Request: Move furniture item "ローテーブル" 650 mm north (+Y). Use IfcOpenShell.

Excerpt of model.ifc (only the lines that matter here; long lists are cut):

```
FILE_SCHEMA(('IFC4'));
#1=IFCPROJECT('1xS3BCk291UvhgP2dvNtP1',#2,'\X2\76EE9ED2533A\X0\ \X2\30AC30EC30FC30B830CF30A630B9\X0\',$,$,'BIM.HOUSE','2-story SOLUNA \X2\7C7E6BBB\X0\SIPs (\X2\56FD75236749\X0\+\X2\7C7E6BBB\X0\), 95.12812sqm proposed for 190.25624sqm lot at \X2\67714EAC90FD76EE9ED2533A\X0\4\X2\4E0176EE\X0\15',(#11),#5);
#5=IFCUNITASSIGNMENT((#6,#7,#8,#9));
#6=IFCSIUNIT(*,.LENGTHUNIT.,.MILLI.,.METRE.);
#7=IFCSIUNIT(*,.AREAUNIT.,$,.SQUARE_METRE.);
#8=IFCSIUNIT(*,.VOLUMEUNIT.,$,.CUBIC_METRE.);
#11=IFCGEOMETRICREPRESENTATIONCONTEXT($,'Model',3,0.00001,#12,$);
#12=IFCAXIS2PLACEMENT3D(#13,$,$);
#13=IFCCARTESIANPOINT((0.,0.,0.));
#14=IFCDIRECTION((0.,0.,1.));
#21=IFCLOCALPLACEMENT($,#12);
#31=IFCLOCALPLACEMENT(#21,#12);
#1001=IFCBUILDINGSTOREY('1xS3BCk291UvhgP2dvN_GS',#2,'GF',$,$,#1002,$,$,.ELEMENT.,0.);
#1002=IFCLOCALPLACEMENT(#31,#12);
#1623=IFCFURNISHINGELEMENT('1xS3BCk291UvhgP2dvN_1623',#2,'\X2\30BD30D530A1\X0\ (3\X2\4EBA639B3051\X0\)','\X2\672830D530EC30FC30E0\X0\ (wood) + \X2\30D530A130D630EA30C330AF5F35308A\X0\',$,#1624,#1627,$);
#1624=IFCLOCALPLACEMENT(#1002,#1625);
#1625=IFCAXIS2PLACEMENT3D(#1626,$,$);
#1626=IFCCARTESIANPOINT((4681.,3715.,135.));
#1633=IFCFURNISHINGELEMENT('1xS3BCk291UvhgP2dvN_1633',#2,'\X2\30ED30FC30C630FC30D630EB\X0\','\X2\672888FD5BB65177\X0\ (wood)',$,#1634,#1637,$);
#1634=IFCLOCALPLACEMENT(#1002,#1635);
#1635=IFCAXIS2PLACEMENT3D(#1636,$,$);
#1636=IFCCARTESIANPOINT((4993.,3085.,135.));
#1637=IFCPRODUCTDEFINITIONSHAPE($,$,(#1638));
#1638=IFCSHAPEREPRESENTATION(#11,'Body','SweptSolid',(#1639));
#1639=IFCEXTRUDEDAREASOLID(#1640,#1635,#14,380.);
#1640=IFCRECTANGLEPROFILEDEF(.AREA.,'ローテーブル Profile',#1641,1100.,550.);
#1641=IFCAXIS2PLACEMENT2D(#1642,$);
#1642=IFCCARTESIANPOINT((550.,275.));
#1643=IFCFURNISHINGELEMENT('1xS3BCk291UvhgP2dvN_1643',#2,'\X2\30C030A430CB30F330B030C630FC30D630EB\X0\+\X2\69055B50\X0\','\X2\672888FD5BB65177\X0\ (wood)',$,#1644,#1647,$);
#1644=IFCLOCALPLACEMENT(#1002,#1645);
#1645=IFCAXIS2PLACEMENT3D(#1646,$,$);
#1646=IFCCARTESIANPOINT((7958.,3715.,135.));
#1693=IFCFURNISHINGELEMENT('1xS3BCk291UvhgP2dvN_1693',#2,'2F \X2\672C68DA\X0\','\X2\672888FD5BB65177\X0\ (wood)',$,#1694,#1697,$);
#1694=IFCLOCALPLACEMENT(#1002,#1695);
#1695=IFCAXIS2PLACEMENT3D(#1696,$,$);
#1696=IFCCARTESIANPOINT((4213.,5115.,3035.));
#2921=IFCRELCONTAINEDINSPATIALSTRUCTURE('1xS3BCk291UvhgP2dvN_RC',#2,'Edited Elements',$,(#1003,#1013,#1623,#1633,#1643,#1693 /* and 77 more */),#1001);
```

```python
import ifcopenshell
import ifcopenshell.api.geometry
import ifcopenshell.util.placement
import ifcopenshell.util.unit

model = ifcopenshell.open("model.ifc")
unit_scale = ifcopenshell.util.unit.calculate_unit_scale(model)

item = model.by_guid("1xS3BCk291UvhgP2dvN_1633")
matrix = ifcopenshell.util.placement.get_local_placement(item.ObjectPlacement)
matrix[1, 3] += 0.65 / unit_scale
ifcopenshell.api.geometry.edit_object_placement(model, product=item, matrix=matrix, is_si=False)

print(ifcopenshell.util.placement.get_local_placement(item.ObjectPlacement).round(3) + 0.0)

model.write("model_edited.ifc")
```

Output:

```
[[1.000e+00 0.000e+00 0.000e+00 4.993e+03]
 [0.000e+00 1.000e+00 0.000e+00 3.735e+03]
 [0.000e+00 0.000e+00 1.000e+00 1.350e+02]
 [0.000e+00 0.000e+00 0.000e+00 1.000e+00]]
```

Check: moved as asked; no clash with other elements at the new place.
